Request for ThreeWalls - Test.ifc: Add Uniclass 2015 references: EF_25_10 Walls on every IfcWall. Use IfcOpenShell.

First a look at what the model holds.

```python
import ifcopenshell

model = ifcopenshell.open("ThreeWalls - Test.ifc")
print(model.schema)
print("classifications:", [c.Name for c in model.by_type("IfcClassification")])
for ifc_class in ("IfcDoor", "IfcRoof", "IfcStair", "IfcWall", "IfcWindow"):
    print(ifc_class, len(model.by_type(ifc_class)))
```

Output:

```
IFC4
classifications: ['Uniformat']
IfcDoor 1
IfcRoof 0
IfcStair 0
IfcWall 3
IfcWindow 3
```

```python
import ifcopenshell
import ifcopenshell.api.classification

model = ifcopenshell.open("ThreeWalls - Test.ifc")

system = ifcopenshell.api.classification.add_classification(model, classification="Uniclass 2015")

codes = {
    "IfcWall": ("EF_25_10", "Walls"),
}
for ifc_class, (code, name) in codes.items():
    products = model.by_type(ifc_class)
    ifcopenshell.api.classification.add_reference(
        model, products=products, classification=system, identification=code, name=name
    )
    print(code, len(products))

model.write("ThreeWalls - Test_rev.ifc")
```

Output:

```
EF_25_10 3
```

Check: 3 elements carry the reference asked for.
